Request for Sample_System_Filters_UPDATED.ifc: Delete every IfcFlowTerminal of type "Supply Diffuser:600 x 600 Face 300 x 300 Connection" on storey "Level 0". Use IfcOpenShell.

First a look at what the model holds.

```python
import ifcopenshell
import ifcopenshell.util.element

model = ifcopenshell.open("Sample_System_Filters_UPDATED.ifc")
print(model.schema)
storey = next(s for s in model.by_type("IfcBuildingStorey") if s.Name == "Level 0")
terminals = [e for e in ifcopenshell.util.element.get_decomposition(storey) if e.is_a("IfcFlowTerminal")]
seen = {}
for e in terminals:
    element_type = ifcopenshell.util.element.get_type(e)
    name = element_type.Name if element_type not in (None, e) else None
    seen[name] = seen.get(name, 0) + 1
for name, count in sorted(seen.items(), key=str):
    print(count, "x", name)
```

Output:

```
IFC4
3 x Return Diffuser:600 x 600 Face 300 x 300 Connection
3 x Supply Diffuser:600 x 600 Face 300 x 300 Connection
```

```python
import ifcopenshell
import ifcopenshell.api.root
import ifcopenshell.util.element

model = ifcopenshell.open("Sample_System_Filters_UPDATED.ifc")

storey = next(s for s in model.by_type("IfcBuildingStorey") if s.Name == "Level 0")
terminals = [e for e in ifcopenshell.util.element.get_decomposition(storey) if e.is_a("IfcFlowTerminal")]
targets = [e for e in terminals if (t := ifcopenshell.util.element.get_type(e)) not in (None, e) and t.Name == "Supply Diffuser:600 x 600 Face 300 x 300 Connection"]

for e in targets:
    ifcopenshell.api.root.remove_product(model, product=e)
print(len(targets), "removed")

model.write("Sample_System_Filters_UPDATED_updated.ifc")
```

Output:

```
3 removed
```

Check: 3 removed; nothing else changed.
